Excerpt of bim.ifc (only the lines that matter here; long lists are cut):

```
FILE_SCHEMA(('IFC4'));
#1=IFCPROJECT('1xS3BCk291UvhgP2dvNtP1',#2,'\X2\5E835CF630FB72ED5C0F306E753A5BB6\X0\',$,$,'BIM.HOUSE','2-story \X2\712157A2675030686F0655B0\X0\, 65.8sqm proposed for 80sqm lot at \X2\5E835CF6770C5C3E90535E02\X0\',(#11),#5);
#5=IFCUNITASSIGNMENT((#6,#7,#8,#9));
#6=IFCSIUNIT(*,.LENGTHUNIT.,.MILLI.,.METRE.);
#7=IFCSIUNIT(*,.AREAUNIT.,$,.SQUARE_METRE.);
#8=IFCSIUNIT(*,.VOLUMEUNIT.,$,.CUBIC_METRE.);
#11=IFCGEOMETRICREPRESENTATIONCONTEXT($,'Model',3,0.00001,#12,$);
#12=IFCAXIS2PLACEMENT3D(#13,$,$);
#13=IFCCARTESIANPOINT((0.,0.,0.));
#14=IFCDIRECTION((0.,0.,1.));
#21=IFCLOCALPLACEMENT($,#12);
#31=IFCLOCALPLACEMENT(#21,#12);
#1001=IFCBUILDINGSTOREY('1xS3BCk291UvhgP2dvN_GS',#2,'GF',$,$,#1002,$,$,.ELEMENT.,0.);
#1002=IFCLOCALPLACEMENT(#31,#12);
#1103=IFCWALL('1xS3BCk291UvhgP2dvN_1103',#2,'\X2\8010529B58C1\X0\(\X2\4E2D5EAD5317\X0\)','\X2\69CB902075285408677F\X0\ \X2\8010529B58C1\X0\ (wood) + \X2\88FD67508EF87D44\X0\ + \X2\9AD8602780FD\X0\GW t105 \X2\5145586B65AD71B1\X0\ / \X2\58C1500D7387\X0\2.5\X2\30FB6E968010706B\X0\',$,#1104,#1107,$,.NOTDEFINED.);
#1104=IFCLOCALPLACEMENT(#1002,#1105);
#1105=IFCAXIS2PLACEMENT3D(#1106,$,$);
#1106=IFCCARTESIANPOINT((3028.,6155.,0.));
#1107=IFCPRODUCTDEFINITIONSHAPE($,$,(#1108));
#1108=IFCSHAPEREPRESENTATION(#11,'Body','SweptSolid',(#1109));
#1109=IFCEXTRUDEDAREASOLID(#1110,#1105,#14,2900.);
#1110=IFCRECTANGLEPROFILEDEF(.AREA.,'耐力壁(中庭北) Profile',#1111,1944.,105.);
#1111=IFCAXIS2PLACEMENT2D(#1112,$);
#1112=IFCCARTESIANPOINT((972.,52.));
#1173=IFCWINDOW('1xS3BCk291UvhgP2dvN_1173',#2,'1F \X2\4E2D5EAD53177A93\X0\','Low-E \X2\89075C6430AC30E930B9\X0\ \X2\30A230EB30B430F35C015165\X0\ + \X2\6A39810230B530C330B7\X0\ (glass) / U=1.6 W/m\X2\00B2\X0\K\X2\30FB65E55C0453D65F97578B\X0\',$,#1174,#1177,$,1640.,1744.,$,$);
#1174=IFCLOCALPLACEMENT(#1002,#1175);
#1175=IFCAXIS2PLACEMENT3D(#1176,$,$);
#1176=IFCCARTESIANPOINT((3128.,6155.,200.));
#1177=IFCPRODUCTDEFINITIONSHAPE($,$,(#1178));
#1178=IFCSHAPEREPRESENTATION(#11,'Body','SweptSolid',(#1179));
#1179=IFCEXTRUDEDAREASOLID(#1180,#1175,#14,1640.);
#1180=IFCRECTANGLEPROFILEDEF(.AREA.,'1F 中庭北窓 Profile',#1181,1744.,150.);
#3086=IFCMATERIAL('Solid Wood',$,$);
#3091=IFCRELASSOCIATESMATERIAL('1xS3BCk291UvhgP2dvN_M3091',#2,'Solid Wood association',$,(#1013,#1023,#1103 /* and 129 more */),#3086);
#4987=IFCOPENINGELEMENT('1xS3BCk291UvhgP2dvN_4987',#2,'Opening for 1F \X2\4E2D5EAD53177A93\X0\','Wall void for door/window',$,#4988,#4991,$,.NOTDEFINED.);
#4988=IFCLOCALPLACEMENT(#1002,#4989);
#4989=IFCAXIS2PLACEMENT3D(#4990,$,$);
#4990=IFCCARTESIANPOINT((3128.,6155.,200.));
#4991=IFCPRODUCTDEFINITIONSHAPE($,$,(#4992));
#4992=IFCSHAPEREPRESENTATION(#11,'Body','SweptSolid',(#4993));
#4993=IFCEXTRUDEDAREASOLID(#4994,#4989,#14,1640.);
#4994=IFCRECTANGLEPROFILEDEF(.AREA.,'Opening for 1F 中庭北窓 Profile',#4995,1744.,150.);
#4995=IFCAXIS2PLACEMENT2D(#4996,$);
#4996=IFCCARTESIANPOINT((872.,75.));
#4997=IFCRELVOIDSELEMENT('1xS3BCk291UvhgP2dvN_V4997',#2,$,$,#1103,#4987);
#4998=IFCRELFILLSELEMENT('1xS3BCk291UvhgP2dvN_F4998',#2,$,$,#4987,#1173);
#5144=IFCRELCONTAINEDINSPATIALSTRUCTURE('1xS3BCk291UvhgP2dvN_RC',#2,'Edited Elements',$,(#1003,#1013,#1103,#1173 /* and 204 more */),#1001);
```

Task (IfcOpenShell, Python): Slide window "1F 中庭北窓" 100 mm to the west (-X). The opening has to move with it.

```python
import ifcopenshell
import ifcopenshell.api.geometry
import ifcopenshell.util.placement
import ifcopenshell.util.unit

model = ifcopenshell.open("bim.ifc")
unit_scale = ifcopenshell.util.unit.calculate_unit_scale(model)

window = model.by_id(1173)
opening = window.FillsVoids[0].RelatingOpeningElement
wall = opening.VoidsElements[0].RelatingBuildingElement

wall_matrix = ifcopenshell.util.placement.get_local_placement(wall.ObjectPlacement)
shift = wall_matrix[:3, 0] * -0.1 / unit_scale
before = ifcopenshell.util.placement.get_local_placement(window.ObjectPlacement)[:3, 3].copy()

# The window is not placed relative to its opening, so move both.
for product in (opening, window):
    matrix = ifcopenshell.util.placement.get_local_placement(product.ObjectPlacement)
    matrix[:3, 3] += shift
    ifcopenshell.api.geometry.edit_object_placement(model, product=product, matrix=matrix, is_si=False)

after = ifcopenshell.util.placement.get_local_placement(window.ObjectPlacement)[:3, 3]
print("window moved by", (after - before).round(3) + 0.0)

model.write("bim-out.ifc")
```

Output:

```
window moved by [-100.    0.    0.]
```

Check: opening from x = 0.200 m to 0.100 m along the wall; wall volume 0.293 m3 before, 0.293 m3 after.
